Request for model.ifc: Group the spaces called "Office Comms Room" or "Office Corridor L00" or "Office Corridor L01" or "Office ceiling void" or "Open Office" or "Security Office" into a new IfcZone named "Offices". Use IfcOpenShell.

First a look at what the model holds.

```python
import ifcopenshell

model = ifcopenshell.open("model.ifc")
print(model.schema)
seen = {}
for space in model.by_type("IfcSpace"):
    seen[space.LongName] = seen.get(space.LongName, 0) + 1
for name, count in sorted(seen.items(), key=str):
    print(count, "x", name)
print("zones:", [z.Name for z in model.by_type("IfcZone")][:20])
```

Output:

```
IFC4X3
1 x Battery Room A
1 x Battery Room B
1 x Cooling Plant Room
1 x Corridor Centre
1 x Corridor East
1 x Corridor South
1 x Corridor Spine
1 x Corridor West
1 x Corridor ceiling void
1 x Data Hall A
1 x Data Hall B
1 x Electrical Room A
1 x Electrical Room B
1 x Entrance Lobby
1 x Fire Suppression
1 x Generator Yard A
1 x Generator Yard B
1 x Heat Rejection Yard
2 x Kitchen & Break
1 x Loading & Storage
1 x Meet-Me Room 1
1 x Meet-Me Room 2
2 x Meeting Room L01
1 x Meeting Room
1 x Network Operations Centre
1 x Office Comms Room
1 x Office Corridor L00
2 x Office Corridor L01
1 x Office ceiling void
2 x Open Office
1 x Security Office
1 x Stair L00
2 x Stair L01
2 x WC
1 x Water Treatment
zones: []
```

```python
import ifcopenshell
import ifcopenshell.api.group
import ifcopenshell.api.root

model = ifcopenshell.open("model.ifc")

names = {"Office Comms Room", "Office Corridor L00", "Office Corridor L01", "Office ceiling void", "Open Office", "Security Office"}
spaces = [s for s in model.by_type("IfcSpace") if s.LongName in names]

zone = ifcopenshell.api.root.create_entity(model, ifc_class="IfcZone", name="Offices")
ifcopenshell.api.group.assign_group(model, products=spaces, group=zone)
print(len(spaces), "spaces in", zone.Name)

model.write("model_v2.ifc")
```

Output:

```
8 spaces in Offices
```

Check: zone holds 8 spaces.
